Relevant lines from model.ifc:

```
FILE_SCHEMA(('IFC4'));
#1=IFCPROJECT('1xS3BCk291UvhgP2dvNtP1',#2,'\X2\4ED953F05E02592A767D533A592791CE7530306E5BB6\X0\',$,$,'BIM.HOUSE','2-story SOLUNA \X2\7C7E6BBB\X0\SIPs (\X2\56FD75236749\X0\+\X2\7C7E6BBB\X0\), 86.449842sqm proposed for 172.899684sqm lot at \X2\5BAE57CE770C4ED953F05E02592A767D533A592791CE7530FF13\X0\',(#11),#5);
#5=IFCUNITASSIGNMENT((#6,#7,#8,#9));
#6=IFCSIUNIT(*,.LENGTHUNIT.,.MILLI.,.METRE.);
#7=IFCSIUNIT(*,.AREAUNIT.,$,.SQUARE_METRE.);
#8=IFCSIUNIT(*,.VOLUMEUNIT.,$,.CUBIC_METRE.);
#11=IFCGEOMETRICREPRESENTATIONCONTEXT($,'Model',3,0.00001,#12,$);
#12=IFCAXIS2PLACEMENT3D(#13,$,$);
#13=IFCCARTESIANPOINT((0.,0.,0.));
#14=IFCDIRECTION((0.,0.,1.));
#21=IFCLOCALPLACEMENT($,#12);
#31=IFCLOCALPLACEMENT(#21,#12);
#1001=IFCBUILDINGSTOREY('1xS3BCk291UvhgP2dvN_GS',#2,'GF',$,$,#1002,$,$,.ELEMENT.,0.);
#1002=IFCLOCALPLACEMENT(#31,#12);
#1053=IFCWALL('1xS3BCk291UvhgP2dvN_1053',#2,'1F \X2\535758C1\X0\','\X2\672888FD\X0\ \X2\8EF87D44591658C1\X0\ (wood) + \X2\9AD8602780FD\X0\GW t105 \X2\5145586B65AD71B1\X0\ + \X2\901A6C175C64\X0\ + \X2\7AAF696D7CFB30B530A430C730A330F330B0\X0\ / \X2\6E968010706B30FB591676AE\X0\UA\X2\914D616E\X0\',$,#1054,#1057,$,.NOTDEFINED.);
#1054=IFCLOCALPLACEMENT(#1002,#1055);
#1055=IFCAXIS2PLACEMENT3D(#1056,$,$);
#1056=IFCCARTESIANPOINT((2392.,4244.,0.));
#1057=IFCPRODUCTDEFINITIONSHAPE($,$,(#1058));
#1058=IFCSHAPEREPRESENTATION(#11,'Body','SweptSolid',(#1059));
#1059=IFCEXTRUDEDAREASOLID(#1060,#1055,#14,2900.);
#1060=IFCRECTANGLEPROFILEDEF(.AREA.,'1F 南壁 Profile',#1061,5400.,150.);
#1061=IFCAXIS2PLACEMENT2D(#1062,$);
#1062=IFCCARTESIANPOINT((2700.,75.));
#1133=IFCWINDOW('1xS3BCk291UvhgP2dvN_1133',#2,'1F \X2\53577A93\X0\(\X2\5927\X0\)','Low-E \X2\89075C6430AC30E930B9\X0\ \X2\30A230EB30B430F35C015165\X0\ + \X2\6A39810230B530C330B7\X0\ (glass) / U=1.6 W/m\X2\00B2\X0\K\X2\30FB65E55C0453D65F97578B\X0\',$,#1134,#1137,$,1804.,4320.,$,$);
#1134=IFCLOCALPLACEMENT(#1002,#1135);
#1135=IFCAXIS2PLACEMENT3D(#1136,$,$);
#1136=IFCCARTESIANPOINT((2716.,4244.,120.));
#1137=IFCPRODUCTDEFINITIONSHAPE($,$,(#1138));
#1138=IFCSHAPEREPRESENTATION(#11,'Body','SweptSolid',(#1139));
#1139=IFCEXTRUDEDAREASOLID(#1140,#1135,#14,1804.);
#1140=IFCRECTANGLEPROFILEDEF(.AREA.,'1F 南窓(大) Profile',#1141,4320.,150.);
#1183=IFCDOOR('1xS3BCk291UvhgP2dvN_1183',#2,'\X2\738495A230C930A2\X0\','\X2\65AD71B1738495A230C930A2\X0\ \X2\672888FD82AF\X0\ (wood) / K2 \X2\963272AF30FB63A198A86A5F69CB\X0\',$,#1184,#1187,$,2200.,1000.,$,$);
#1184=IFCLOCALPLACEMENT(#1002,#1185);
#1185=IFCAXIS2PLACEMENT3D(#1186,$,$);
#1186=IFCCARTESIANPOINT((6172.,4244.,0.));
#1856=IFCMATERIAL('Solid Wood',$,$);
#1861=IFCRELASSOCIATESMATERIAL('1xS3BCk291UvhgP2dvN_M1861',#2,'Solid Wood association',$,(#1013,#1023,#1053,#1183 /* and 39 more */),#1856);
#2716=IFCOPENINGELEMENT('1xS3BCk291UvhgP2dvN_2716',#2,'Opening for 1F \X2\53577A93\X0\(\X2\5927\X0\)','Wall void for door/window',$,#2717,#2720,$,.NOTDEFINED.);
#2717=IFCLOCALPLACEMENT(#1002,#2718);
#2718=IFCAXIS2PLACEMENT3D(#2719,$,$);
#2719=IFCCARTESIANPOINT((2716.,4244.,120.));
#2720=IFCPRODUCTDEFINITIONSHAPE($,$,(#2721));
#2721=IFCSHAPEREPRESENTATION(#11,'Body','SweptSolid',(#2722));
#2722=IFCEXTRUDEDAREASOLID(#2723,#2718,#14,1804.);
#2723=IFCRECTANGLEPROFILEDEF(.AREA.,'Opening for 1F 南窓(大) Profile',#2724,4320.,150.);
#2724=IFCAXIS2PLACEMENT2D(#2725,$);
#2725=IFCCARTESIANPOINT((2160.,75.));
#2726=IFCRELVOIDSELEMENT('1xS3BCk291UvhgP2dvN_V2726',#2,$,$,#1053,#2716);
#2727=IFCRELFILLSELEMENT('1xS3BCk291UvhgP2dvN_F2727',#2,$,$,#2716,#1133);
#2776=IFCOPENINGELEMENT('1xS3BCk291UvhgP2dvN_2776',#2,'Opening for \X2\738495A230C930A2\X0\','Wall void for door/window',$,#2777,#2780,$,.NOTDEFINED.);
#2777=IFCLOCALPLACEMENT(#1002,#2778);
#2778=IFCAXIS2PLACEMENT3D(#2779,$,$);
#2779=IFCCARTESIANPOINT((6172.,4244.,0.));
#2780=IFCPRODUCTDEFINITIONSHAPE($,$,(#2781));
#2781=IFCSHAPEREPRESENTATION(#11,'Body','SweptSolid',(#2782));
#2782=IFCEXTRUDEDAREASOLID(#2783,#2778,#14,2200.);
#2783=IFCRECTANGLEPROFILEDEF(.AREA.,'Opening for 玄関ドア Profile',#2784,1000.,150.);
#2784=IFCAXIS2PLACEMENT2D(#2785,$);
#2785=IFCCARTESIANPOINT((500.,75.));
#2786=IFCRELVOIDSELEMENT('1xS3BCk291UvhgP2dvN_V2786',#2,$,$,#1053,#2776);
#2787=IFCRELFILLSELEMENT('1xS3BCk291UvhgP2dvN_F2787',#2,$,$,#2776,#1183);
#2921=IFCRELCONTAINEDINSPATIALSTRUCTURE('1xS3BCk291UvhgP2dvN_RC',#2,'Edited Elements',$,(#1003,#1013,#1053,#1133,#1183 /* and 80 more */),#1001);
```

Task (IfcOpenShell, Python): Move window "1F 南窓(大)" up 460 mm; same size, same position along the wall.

```python
import numpy as np
import ifcopenshell
import ifcopenshell.api.geometry
import ifcopenshell.util.placement
import ifcopenshell.util.unit

model = ifcopenshell.open("model.ifc")
unit_scale = ifcopenshell.util.unit.calculate_unit_scale(model)

window = model.by_guid("1xS3BCk291UvhgP2dvN_1133")
opening = window.FillsVoids[0].RelatingOpeningElement
dz = 460.0

shift = np.array([0.0, 0.0, dz])
# The window is not placed relative to its opening, so move both.
for product in (opening, window):
    matrix = ifcopenshell.util.placement.get_local_placement(product.ObjectPlacement)
    matrix[:3, 3] += shift
    ifcopenshell.api.geometry.edit_object_placement(model, product=product, matrix=matrix, is_si=False)

print(f"moved by {dz * unit_scale:+.3f} m")

model.write("model_rev.ifc")
```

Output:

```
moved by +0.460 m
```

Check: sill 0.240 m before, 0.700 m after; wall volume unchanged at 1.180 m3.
